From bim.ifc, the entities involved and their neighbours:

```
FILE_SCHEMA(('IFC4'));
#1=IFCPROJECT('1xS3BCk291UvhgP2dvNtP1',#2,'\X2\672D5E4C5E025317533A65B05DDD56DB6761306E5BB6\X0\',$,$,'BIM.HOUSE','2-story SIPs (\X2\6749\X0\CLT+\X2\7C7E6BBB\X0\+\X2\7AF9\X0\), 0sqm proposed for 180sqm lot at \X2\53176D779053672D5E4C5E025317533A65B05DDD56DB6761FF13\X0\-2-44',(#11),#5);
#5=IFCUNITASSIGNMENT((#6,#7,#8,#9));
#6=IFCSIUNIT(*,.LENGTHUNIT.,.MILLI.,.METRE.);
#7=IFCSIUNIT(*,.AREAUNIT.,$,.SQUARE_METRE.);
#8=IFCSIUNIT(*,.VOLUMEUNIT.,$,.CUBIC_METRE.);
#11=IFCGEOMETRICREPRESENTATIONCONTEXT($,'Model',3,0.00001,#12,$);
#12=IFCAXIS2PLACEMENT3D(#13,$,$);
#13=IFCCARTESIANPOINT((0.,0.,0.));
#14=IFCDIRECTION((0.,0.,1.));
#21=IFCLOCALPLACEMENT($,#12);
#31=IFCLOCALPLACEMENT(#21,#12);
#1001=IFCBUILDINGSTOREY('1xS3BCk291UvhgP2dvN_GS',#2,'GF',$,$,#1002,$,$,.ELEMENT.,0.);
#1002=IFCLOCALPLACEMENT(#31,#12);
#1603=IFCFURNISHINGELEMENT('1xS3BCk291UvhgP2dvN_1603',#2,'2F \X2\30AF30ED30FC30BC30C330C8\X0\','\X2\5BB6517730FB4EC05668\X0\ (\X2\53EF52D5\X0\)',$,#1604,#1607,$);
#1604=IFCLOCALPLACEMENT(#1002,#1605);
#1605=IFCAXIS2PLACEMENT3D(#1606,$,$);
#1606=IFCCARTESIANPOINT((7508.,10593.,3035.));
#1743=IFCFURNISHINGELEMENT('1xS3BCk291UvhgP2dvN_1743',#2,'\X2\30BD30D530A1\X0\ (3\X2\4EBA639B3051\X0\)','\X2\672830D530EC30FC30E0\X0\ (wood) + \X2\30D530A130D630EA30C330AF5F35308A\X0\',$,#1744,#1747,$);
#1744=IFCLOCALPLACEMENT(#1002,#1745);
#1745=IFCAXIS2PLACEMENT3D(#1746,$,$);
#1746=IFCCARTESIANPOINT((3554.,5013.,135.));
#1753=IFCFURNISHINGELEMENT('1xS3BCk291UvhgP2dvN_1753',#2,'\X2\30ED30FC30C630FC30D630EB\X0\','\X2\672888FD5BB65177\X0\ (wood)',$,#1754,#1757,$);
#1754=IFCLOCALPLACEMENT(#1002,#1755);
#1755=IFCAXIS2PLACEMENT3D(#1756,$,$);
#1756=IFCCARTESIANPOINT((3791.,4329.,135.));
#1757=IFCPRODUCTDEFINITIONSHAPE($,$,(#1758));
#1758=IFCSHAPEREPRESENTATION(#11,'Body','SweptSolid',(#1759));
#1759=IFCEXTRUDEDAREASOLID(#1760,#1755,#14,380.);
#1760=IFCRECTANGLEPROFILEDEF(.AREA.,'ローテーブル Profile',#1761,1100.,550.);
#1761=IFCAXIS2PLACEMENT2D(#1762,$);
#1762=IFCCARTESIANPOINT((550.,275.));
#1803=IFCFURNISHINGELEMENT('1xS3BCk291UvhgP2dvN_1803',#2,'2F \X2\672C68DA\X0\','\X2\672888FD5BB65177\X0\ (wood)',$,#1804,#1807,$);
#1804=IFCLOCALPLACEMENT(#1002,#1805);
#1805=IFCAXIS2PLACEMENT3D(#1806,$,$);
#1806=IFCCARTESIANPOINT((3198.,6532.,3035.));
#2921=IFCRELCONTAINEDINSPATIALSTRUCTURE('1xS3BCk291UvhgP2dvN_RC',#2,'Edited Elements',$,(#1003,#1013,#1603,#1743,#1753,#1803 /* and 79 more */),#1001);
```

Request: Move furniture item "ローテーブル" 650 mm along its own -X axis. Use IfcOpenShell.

```python
import ifcopenshell
import ifcopenshell.api.geometry
import ifcopenshell.util.placement
import ifcopenshell.util.unit

model = ifcopenshell.open("bim.ifc")
unit_scale = ifcopenshell.util.unit.calculate_unit_scale(model)

item = model.by_guid("1xS3BCk291UvhgP2dvN_1753")
matrix = ifcopenshell.util.placement.get_local_placement(item.ObjectPlacement)
matrix[:3, 3] -= matrix[:3, 0] * 0.65 / unit_scale
ifcopenshell.api.geometry.edit_object_placement(model, product=item, matrix=matrix, is_si=False)

print(ifcopenshell.util.placement.get_local_placement(item.ObjectPlacement).round(3) + 0.0)

model.write("bim_v2.ifc")
```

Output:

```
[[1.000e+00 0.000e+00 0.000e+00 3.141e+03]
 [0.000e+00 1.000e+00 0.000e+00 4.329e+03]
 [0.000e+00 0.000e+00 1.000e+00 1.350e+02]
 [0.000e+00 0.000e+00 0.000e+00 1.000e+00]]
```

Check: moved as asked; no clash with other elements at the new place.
